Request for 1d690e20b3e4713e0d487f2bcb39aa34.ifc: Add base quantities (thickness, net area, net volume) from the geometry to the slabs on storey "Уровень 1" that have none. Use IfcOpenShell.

First a look at what the model holds.

```python
import ifcopenshell
import ifcopenshell.util.element
import ifcopenshell.util.unit

model = ifcopenshell.open("1d690e20b3e4713e0d487f2bcb39aa34.ifc")
print(model.schema)
for unit_type in ("LENGTHUNIT", "AREAUNIT", "VOLUMEUNIT"):
    print(unit_type, ifcopenshell.util.unit.calculate_unit_scale(model, unit_type))
storey = next(s for s in model.by_type("IfcBuildingStorey") if s.Name == "Уровень 1")
slabs = [e for e in ifcopenshell.util.element.get_decomposition(storey) if e.is_a("IfcSlab")]
for e in sorted(slabs, key=lambda e: e.id()):
    print(e.id(), e.is_a(), e.Name, list(ifcopenshell.util.element.get_psets(e, qtos_only=True)), sep=" | ")
```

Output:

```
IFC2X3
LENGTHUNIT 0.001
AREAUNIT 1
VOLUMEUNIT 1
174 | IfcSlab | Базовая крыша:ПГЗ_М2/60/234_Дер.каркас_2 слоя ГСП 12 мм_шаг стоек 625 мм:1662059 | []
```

```python
import ifcopenshell
import ifcopenshell.api.pset
import ifcopenshell.geom
import ifcopenshell.util.element
import ifcopenshell.util.shape
import ifcopenshell.util.unit

model = ifcopenshell.open("1d690e20b3e4713e0d487f2bcb39aa34.ifc")
unit_scale = ifcopenshell.util.unit.calculate_unit_scale(model)
area_scale = ifcopenshell.util.unit.calculate_unit_scale(model, "AREAUNIT")
volume_scale = ifcopenshell.util.unit.calculate_unit_scale(model, "VOLUMEUNIT")
settings = ifcopenshell.geom.settings()

storey = next(s for s in model.by_type("IfcBuildingStorey") if s.Name == "Уровень 1")
slabs = [e for e in ifcopenshell.util.element.get_decomposition(storey) if e.is_a("IfcSlab")]

for e in sorted(slabs, key=lambda e: e.id()):
    if ifcopenshell.util.element.get_psets(e, qtos_only=True, should_inherit=False):
        continue
    # Geometry comes back in metres, in the element's own axes.
    shape = ifcopenshell.geom.create_shape(settings, e)
    values = {
        "Width": ifcopenshell.util.shape.get_z(shape.geometry) / unit_scale,
        "NetArea": ifcopenshell.util.shape.get_footprint_area(shape.geometry) / area_scale,
        "NetVolume": ifcopenshell.util.shape.get_volume(shape.geometry) / volume_scale,
    }
    qto = ifcopenshell.api.pset.add_qto(model, product=e, name="BaseQuantities")
    ifcopenshell.api.pset.edit_qto(model, qto=qto, properties=values)
    print(e.id(), {k: round(v, 3) for k, v in values.items()})

model.write("1d690e20b3e4713e0d487f2bcb39aa34-out.ifc")
```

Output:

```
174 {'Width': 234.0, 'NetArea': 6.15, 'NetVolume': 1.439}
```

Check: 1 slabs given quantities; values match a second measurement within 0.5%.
